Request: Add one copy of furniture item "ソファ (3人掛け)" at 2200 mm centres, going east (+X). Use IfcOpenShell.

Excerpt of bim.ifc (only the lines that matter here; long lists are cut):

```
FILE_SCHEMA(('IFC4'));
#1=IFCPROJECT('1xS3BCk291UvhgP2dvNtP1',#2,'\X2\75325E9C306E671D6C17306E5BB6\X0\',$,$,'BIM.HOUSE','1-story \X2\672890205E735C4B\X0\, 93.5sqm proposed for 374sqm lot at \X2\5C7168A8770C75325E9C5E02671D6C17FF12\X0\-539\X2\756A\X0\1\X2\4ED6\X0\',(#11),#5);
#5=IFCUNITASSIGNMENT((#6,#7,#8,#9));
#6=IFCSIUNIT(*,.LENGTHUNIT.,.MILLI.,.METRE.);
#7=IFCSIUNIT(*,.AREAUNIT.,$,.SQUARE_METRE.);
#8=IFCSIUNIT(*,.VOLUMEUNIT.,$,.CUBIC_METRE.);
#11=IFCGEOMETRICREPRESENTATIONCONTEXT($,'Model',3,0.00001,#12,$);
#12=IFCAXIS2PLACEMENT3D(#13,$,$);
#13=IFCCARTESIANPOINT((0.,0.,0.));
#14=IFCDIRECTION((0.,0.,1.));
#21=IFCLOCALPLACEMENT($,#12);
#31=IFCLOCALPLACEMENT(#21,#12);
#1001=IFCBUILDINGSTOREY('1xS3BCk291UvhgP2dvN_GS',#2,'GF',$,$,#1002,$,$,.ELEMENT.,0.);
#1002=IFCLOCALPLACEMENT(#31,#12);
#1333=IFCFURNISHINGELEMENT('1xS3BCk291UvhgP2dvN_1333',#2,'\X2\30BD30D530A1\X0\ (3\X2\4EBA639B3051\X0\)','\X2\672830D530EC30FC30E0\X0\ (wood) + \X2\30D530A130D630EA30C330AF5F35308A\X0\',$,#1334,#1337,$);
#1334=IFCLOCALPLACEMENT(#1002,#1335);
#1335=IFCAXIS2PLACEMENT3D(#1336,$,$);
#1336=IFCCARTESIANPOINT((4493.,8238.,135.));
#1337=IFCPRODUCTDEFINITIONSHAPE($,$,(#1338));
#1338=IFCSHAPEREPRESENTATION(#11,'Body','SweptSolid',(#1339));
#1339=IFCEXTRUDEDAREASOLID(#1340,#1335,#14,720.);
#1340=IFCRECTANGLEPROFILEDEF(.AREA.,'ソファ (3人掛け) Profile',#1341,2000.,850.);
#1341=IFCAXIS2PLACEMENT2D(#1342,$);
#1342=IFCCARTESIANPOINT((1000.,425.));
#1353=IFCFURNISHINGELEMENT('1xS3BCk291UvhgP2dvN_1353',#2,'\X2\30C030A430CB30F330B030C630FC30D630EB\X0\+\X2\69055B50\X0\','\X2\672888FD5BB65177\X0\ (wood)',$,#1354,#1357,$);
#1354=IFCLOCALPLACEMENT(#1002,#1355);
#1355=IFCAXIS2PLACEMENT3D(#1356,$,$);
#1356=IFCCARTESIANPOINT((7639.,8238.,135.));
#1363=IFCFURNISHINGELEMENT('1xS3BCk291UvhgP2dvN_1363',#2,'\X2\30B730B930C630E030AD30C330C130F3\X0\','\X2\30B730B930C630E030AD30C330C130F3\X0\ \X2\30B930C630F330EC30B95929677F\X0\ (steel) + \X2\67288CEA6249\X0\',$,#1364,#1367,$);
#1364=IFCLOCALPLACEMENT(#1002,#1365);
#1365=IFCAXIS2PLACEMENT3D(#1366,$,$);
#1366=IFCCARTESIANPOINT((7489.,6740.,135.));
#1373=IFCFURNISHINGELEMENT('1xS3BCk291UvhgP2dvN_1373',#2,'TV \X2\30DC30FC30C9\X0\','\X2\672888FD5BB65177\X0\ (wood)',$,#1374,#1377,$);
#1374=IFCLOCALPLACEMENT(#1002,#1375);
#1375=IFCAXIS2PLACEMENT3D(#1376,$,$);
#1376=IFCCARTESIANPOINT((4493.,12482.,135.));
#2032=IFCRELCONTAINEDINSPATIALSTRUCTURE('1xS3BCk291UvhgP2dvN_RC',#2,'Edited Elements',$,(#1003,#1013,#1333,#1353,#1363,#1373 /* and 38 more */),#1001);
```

```python
import numpy as np
import ifcopenshell
import ifcopenshell.api.geometry
import ifcopenshell.api.root
import ifcopenshell.util.element
import ifcopenshell.util.placement

model = ifcopenshell.open("bim.ifc")


def reuse_history(source, copy):
    """copy_class also copies each property set's owner history, people and application; keep the originals."""
    for rel in copy.IsDefinedBy:
        if rel.is_a("IfcRelDefinesByProperties") and (history := rel.RelatingPropertyDefinition.OwnerHistory):
            rel.RelatingPropertyDefinition.OwnerHistory = source.OwnerHistory
            ifcopenshell.util.element.remove_deep2(model, history)


source = model.by_guid("1xS3BCk291UvhgP2dvN_1333")
base = ifcopenshell.util.placement.get_local_placement(source.ObjectPlacement)
step = np.array([1.0, 0.0, 0.0]) * 2200.0

for i in range(1, 2):
    copy = ifcopenshell.api.root.copy_class(model, product=source)
    copy.Representation = ifcopenshell.util.element.copy_deep(
        model, source.Representation, exclude=["IfcGeometricRepresentationContext", "IfcRepresentationMap"]
    )
    reuse_history(source, copy)
    matrix = base.copy()
    matrix[:3, 3] += i * step
    print("added at", matrix[:3, 3].round(3) + 0.0)
    ifcopenshell.api.geometry.edit_object_placement(model, product=copy, matrix=matrix, is_si=False)

model.write("bim_updated.ifc")
```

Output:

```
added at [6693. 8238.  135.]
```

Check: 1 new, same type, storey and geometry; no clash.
